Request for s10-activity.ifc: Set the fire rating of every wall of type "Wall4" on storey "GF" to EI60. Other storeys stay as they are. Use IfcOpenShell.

First a look at what the model holds.

```python
import ifcopenshell
import ifcopenshell.util.element

model = ifcopenshell.open("s10-activity.ifc")
print(model.schema)
storey = next(s for s in model.by_type("IfcBuildingStorey") if s.Name == "GF")
walls = [e for e in ifcopenshell.util.element.get_decomposition(storey) if e.is_a("IfcWall")]
seen = {}
for e in walls:
    element_type = ifcopenshell.util.element.get_type(e)
    key = (element_type.Name if element_type != e and element_type else None, ifcopenshell.util.element.get_pset(e, "Pset_WallCommon", "FireRating"))
    seen[key] = seen.get(key, 0) + 1
for (name, value), count in sorted(seen.items(), key=str):
    print(count, "x", name, "|", value)
```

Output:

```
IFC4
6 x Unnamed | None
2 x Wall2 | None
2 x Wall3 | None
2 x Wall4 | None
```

```python
import ifcopenshell
import ifcopenshell.api.pset
import ifcopenshell.util.element

model = ifcopenshell.open("s10-activity.ifc")

storey = next(s for s in model.by_type("IfcBuildingStorey") if s.Name == "GF")
walls = [e for e in ifcopenshell.util.element.get_decomposition(storey) if e.is_a("IfcWall")]

count = 0
for e in walls:
    element_type = ifcopenshell.util.element.get_type(e)
    if element_type in (None, e) or element_type.Name != "Wall4":
        continue
    # add_pset returns the element's existing set when there is one.
    pset = ifcopenshell.api.pset.add_pset(model, product=e, name="Pset_WallCommon")
    ifcopenshell.api.pset.edit_pset(model, pset=pset, properties={"FireRating": "EI60"})
    count += 1

print(count, "walls updated")

model.write("s10-activity_edited.ifc")
```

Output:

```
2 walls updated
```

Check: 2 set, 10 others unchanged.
